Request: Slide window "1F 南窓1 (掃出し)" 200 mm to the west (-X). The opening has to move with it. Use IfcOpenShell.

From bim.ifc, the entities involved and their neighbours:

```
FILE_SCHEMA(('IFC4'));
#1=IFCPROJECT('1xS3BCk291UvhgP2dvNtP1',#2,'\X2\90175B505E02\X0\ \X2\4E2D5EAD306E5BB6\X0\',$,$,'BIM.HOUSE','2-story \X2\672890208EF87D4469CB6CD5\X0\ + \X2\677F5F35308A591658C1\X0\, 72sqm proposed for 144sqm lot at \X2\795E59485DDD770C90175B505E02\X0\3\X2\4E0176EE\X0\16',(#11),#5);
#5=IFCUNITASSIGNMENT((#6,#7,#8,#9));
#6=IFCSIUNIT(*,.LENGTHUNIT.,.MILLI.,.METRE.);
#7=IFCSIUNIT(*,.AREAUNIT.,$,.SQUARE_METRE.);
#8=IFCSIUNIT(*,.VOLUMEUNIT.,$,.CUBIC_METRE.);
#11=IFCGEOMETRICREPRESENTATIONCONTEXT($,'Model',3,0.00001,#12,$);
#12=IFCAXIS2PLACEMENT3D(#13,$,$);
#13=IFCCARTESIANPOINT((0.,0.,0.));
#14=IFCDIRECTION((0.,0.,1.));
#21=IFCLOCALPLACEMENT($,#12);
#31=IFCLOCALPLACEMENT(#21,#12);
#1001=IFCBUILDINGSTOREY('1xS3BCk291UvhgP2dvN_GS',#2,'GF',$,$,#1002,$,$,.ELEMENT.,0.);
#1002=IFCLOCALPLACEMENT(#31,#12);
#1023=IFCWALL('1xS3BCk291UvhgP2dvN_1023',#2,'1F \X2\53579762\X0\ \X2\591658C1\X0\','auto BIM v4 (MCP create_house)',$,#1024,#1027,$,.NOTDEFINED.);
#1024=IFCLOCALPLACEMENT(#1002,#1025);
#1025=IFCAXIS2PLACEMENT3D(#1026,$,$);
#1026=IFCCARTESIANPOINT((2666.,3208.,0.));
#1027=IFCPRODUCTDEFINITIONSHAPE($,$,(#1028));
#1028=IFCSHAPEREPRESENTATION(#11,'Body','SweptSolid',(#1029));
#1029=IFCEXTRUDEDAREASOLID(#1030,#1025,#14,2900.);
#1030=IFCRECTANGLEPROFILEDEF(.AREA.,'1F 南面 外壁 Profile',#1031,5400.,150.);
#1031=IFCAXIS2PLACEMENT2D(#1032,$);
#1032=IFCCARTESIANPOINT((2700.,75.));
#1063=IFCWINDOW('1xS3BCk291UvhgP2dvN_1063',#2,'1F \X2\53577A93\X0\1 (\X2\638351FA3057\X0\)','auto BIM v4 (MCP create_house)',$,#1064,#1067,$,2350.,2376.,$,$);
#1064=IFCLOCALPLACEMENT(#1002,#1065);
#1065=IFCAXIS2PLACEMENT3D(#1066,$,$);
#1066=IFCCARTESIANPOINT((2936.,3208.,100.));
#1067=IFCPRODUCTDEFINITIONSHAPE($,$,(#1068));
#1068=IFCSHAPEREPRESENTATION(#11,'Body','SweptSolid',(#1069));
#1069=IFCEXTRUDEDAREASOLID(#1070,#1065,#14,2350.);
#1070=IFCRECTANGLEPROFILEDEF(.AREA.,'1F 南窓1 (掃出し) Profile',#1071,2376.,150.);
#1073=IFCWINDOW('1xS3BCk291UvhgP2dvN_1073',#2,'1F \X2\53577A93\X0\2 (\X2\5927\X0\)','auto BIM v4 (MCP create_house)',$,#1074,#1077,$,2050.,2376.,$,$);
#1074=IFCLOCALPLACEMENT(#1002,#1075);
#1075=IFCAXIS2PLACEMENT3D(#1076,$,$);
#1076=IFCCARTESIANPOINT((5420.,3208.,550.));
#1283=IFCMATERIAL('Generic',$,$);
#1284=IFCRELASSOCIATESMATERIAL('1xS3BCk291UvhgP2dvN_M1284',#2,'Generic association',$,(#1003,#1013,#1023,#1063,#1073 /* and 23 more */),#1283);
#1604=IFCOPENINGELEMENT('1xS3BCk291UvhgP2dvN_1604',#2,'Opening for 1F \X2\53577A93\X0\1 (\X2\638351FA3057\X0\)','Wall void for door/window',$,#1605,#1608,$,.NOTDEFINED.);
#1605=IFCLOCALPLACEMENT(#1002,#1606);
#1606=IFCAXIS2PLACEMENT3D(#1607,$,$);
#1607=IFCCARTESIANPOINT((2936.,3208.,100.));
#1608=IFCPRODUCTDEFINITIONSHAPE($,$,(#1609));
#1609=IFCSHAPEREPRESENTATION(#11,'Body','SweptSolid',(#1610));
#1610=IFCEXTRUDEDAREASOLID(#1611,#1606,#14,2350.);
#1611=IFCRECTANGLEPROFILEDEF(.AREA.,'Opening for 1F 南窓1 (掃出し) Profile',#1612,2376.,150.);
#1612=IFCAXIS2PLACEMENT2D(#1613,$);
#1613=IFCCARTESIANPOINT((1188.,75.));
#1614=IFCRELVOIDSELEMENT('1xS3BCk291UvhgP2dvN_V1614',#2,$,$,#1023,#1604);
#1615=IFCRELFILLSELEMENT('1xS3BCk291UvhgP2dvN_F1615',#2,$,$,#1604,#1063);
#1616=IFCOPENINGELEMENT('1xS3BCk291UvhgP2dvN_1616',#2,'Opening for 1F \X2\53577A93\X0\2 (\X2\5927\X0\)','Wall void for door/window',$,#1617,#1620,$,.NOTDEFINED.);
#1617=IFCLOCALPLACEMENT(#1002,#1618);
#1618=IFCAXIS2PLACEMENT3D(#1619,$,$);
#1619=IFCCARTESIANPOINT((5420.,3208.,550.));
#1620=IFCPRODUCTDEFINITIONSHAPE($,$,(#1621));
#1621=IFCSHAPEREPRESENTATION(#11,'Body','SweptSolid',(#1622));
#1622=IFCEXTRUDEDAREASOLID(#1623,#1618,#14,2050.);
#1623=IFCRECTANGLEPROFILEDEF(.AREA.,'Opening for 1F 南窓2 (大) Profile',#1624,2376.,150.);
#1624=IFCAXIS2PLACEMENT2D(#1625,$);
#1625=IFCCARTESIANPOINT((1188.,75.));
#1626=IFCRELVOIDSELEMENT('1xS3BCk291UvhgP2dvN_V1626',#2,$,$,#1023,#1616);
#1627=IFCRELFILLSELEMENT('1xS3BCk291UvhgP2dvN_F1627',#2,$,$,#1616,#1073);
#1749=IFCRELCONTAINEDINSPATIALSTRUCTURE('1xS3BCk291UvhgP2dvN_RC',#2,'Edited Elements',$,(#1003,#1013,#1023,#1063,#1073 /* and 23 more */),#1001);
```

```python
import ifcopenshell
import ifcopenshell.api.geometry
import ifcopenshell.util.placement

model = ifcopenshell.open("bim.ifc")

window = model.by_guid("1xS3BCk291UvhgP2dvN_1063")
opening = window.FillsVoids[0].RelatingOpeningElement
wall = opening.VoidsElements[0].RelatingBuildingElement

wall_matrix = ifcopenshell.util.placement.get_local_placement(wall.ObjectPlacement)
shift = wall_matrix[:3, 0] * -200.0
before = ifcopenshell.util.placement.get_local_placement(window.ObjectPlacement)[:3, 3].copy()

# The window is not placed relative to its opening, so move both.
for product in (opening, window):
    matrix = ifcopenshell.util.placement.get_local_placement(product.ObjectPlacement)
    matrix[:3, 3] += shift
    ifcopenshell.api.geometry.edit_object_placement(model, product=product, matrix=matrix, is_si=False)

after = ifcopenshell.util.placement.get_local_placement(window.ObjectPlacement)[:3, 3]
print("window moved by", (after - before).round(3) + 0.0)

model.write("bim-out.ifc")
```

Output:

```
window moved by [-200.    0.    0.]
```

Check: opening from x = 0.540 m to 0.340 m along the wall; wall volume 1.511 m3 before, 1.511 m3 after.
